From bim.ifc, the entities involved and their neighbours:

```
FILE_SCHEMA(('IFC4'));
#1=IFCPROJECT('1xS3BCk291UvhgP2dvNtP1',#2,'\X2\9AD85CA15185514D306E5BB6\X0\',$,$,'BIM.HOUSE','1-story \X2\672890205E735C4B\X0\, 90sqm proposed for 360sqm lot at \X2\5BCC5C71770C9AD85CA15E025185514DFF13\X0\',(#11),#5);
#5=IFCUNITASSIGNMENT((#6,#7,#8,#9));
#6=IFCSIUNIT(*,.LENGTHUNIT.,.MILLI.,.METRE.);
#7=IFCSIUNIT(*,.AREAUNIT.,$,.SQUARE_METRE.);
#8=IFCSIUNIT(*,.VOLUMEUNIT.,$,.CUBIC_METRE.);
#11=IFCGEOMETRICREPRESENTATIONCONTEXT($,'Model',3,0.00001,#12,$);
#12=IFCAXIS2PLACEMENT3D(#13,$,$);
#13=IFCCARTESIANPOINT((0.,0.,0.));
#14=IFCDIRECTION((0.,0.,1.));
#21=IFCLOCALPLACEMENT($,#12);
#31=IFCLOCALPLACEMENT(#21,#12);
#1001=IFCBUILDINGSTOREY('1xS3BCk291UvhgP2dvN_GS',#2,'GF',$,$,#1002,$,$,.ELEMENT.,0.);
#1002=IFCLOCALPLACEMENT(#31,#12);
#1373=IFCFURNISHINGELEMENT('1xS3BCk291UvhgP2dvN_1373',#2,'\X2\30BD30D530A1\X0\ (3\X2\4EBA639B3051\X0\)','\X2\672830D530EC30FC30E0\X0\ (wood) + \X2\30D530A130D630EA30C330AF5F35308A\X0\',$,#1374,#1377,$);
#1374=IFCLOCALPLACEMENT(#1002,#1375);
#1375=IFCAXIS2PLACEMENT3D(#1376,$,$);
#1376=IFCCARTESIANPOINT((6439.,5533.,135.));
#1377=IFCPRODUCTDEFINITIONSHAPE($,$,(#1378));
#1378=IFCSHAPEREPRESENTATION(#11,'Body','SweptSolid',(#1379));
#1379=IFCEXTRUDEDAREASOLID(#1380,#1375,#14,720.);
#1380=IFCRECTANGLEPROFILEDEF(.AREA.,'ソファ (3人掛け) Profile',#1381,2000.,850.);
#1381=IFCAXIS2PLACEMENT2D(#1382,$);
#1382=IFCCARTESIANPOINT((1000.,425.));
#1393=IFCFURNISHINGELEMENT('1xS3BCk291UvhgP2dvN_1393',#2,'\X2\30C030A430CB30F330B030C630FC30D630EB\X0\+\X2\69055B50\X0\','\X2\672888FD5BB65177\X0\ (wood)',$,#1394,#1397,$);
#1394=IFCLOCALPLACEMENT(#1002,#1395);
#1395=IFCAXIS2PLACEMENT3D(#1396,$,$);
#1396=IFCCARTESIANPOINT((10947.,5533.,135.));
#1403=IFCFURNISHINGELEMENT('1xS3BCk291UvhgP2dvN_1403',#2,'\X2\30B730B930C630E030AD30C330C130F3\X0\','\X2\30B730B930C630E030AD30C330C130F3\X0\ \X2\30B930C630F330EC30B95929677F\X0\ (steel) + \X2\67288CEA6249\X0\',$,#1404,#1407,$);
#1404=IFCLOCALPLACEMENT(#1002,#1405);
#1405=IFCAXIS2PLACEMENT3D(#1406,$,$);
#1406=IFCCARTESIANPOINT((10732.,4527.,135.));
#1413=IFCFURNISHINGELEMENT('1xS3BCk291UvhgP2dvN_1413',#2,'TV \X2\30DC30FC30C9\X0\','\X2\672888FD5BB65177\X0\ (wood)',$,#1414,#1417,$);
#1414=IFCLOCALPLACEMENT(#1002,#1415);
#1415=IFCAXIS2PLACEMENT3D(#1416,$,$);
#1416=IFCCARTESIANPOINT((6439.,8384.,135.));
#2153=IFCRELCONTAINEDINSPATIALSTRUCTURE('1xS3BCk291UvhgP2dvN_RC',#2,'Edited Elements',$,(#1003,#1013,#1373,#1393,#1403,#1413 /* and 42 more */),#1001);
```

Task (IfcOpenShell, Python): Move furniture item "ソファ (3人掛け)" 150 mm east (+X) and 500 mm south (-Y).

```python
import ifcopenshell
import ifcopenshell.api.geometry
import ifcopenshell.util.placement
import ifcopenshell.util.unit

model = ifcopenshell.open("bim.ifc")
unit_scale = ifcopenshell.util.unit.calculate_unit_scale(model)

item = model.by_guid("1xS3BCk291UvhgP2dvN_1373")
matrix = ifcopenshell.util.placement.get_local_placement(item.ObjectPlacement)
matrix[0, 3] += 0.15 / unit_scale
matrix[1, 3] -= 0.5 / unit_scale
ifcopenshell.api.geometry.edit_object_placement(model, product=item, matrix=matrix, is_si=False)

print(ifcopenshell.util.placement.get_local_placement(item.ObjectPlacement).round(3) + 0.0)

model.write("bim-out.ifc")
```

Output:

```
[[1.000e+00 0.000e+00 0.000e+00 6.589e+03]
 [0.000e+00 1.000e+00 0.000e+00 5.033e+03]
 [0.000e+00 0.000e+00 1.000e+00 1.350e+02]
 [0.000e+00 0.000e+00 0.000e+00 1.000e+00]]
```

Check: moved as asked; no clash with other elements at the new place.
